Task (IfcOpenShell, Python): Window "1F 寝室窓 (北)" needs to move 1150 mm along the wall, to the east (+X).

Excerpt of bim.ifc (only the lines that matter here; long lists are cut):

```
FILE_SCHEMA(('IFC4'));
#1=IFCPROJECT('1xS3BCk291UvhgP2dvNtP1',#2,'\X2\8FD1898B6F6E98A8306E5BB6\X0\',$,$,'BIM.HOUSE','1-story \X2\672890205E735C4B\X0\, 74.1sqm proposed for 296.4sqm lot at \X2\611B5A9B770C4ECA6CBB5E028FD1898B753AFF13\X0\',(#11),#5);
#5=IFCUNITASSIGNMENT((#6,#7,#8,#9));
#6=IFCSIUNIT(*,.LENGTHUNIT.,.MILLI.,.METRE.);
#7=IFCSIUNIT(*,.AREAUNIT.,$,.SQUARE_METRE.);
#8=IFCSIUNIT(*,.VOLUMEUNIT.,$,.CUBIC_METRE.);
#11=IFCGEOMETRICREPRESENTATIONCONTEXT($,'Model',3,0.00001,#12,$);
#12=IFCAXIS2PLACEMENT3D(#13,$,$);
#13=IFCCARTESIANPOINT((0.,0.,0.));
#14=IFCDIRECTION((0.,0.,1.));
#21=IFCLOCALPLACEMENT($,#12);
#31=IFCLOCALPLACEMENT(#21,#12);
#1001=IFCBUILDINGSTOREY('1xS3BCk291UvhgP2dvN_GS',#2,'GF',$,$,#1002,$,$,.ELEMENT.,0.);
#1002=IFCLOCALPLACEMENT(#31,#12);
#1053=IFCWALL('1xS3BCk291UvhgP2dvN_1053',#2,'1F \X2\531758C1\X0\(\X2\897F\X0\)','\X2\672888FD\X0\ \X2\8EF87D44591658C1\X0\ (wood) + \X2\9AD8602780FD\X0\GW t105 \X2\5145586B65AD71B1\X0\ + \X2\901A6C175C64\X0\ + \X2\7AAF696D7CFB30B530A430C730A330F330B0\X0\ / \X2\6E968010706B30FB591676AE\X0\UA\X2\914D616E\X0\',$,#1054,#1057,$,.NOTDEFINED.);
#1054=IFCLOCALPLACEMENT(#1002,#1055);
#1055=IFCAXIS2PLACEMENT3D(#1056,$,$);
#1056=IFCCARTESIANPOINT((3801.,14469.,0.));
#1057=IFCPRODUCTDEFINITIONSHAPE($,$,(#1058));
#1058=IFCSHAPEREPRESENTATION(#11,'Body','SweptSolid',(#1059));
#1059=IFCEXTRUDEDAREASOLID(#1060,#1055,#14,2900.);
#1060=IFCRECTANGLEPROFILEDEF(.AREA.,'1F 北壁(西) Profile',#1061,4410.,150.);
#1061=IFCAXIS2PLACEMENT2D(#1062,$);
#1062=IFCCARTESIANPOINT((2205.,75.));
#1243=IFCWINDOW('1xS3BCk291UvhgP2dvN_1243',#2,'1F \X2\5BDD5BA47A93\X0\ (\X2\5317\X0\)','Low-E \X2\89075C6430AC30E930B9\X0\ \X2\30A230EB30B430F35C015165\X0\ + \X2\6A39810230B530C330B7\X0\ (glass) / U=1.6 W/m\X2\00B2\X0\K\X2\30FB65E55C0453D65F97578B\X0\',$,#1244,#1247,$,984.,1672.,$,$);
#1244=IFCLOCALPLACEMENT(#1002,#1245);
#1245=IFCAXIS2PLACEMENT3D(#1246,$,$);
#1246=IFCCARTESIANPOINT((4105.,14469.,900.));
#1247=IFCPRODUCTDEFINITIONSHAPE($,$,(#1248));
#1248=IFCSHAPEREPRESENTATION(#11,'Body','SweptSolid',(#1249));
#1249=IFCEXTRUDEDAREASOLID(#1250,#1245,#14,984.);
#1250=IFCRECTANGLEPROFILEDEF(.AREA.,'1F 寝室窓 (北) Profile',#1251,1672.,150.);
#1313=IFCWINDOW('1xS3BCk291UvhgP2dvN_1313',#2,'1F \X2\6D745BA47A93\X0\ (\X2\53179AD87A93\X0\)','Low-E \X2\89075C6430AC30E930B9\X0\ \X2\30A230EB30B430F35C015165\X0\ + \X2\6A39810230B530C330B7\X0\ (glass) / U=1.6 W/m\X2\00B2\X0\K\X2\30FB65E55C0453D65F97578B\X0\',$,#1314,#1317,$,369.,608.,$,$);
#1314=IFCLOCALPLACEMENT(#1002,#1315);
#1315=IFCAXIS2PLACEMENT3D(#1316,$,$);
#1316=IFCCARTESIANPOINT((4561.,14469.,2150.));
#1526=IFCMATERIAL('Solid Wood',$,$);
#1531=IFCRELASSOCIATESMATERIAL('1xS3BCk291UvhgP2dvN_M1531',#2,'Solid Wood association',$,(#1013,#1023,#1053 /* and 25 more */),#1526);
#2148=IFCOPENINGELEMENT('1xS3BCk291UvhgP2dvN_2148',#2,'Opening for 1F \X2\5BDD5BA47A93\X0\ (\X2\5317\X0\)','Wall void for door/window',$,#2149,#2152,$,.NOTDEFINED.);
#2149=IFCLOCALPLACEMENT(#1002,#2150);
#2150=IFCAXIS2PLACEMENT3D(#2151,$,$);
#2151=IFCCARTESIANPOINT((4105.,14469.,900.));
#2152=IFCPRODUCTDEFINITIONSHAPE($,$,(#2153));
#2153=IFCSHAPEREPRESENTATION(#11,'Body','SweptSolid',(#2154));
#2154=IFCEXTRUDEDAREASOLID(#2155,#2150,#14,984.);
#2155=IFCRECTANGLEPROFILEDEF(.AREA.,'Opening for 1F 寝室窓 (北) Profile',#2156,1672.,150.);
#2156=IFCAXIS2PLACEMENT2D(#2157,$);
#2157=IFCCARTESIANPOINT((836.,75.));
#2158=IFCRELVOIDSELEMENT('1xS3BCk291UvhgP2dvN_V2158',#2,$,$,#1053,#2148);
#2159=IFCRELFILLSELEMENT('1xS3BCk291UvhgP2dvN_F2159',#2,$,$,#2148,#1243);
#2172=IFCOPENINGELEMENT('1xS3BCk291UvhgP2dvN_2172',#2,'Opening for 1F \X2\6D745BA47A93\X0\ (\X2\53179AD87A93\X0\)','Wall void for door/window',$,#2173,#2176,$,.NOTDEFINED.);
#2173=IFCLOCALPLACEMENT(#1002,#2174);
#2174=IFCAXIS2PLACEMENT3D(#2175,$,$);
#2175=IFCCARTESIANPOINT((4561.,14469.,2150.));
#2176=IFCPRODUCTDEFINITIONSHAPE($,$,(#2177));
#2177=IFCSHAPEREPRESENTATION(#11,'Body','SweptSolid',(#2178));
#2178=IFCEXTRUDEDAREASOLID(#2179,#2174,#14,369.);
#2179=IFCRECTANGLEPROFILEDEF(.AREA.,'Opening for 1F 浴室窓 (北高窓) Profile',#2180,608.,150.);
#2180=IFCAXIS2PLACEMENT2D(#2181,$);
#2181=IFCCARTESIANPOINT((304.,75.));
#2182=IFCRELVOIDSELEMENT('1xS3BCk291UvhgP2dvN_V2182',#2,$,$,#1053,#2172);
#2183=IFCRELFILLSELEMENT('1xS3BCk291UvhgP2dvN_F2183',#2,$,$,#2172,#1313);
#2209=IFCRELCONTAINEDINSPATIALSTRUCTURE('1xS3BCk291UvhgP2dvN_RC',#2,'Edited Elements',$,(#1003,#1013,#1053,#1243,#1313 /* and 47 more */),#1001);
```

```python
import ifcopenshell
import ifcopenshell.api.geometry
import ifcopenshell.util.placement
import ifcopenshell.util.unit

model = ifcopenshell.open("bim.ifc")
unit_scale = ifcopenshell.util.unit.calculate_unit_scale(model)

window = model.by_guid("1xS3BCk291UvhgP2dvN_1243")
opening = window.FillsVoids[0].RelatingOpeningElement
wall = opening.VoidsElements[0].RelatingBuildingElement

wall_matrix = ifcopenshell.util.placement.get_local_placement(wall.ObjectPlacement)
shift = wall_matrix[:3, 0] * 1.15 / unit_scale
before = ifcopenshell.util.placement.get_local_placement(window.ObjectPlacement)[:3, 3].copy()

# The window is not placed relative to its opening, so move both.
for product in (opening, window):
    matrix = ifcopenshell.util.placement.get_local_placement(product.ObjectPlacement)
    matrix[:3, 3] += shift
    ifcopenshell.api.geometry.edit_object_placement(model, product=product, matrix=matrix, is_si=False)

after = ifcopenshell.util.placement.get_local_placement(window.ObjectPlacement)[:3, 3]
print("window moved by", (after - before).round(3) + 0.0)

model.write("bim_edited.ifc")
```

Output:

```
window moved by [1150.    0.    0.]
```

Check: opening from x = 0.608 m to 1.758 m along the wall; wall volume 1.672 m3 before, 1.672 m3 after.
